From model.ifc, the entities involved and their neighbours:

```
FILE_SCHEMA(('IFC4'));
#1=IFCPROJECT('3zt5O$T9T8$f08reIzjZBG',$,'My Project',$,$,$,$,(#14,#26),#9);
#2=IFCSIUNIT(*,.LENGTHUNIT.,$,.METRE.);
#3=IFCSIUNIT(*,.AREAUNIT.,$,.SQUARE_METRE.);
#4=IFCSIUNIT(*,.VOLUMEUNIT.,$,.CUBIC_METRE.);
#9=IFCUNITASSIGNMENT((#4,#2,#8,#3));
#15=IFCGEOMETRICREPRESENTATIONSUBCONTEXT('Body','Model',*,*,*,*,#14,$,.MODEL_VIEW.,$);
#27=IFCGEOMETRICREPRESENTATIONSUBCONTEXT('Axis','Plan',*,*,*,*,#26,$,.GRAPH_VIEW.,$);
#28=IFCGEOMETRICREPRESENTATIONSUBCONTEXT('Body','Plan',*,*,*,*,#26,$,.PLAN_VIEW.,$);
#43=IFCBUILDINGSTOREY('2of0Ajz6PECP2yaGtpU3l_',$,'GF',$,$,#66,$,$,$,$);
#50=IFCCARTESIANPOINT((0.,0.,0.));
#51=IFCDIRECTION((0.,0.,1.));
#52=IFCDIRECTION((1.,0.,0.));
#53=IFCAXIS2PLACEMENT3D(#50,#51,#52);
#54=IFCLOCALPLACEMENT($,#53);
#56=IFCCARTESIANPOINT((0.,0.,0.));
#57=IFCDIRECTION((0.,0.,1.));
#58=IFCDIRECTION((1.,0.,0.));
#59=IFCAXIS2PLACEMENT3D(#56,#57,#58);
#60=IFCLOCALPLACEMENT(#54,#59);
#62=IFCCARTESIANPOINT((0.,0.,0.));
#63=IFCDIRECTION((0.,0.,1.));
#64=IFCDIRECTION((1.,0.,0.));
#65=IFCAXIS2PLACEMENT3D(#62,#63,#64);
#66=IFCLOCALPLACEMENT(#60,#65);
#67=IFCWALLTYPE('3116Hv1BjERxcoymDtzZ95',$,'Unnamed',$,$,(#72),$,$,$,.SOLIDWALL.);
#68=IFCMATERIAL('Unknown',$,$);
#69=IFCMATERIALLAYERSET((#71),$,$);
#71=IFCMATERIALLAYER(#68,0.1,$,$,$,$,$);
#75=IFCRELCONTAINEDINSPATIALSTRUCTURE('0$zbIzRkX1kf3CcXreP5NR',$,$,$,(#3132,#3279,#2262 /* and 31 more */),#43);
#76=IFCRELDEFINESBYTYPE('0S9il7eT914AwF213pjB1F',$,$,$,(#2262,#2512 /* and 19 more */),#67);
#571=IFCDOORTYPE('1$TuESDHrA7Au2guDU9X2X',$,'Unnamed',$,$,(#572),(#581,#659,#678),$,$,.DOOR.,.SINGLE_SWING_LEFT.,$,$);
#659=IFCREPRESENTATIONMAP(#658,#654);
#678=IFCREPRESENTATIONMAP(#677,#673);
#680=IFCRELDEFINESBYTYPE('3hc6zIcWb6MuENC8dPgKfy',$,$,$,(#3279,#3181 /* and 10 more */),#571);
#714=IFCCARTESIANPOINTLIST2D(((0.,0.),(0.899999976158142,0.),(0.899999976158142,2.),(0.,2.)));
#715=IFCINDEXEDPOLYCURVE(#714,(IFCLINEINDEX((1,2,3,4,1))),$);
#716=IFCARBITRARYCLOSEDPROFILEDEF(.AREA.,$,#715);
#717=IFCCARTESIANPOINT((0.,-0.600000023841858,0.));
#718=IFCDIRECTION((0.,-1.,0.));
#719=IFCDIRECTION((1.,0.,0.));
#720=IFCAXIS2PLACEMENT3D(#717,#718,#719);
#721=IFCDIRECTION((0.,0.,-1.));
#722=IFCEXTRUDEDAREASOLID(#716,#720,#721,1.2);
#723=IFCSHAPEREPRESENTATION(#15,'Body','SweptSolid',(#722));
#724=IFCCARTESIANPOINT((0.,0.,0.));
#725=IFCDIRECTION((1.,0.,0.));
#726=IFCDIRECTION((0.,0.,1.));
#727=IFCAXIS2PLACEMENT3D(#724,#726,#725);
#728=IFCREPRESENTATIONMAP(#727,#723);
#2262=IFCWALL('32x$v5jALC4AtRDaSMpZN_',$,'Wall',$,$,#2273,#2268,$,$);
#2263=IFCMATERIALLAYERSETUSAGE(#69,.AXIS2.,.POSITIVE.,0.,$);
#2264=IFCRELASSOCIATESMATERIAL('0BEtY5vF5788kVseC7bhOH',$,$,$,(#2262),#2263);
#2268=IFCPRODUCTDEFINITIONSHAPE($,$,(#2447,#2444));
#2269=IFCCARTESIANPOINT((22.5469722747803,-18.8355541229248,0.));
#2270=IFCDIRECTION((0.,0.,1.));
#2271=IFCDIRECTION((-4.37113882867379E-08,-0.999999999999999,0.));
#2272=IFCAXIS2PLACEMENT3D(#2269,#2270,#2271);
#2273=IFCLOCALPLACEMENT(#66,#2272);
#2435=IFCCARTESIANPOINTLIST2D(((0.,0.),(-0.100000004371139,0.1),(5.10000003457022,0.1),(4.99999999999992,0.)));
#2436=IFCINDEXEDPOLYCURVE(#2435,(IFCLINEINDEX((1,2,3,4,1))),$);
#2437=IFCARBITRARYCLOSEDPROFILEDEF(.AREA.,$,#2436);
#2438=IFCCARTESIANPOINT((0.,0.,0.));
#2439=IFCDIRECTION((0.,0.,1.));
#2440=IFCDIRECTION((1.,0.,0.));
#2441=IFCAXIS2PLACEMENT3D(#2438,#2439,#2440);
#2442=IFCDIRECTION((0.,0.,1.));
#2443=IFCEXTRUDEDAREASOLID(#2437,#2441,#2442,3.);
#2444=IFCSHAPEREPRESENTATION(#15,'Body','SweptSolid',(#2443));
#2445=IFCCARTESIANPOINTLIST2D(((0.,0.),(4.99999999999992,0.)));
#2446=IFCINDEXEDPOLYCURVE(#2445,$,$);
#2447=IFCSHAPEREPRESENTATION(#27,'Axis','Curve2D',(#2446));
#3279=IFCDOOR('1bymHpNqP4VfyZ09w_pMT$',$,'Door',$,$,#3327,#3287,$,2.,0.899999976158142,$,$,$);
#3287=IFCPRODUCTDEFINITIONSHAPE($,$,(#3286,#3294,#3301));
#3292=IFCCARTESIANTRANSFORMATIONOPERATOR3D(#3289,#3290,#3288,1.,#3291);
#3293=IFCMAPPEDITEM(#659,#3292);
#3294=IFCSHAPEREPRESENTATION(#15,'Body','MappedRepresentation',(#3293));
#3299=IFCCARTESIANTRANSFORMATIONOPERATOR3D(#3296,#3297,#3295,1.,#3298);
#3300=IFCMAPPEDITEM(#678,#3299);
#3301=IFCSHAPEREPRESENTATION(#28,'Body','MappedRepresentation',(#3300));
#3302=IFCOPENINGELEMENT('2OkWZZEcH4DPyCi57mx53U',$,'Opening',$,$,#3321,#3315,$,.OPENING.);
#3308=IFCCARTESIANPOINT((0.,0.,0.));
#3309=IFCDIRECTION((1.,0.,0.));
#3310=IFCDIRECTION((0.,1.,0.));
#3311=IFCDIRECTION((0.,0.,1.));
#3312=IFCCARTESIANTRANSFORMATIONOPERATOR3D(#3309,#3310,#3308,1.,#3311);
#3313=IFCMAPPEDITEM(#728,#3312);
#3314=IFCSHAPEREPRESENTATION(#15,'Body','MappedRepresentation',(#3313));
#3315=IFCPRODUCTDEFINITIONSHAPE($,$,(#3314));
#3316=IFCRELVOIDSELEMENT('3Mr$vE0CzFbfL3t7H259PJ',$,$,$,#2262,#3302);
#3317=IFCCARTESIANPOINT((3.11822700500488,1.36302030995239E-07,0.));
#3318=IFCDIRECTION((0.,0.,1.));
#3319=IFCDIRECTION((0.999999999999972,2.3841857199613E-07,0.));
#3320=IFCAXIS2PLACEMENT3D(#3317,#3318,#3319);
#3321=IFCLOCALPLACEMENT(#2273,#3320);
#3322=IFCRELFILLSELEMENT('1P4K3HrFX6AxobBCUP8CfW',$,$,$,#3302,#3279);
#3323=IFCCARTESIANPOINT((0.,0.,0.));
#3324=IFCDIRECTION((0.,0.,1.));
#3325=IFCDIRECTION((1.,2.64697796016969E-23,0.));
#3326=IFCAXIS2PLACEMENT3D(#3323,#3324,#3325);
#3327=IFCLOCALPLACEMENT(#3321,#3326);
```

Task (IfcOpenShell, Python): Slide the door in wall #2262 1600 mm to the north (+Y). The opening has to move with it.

```python
import ifcopenshell
import ifcopenshell.api.geometry
import ifcopenshell.util.placement
import ifcopenshell.util.unit

model = ifcopenshell.open("model.ifc")
unit_scale = ifcopenshell.util.unit.calculate_unit_scale(model)

door = model.by_id(3279)
opening = door.FillsVoids[0].RelatingOpeningElement
wall = opening.VoidsElements[0].RelatingBuildingElement

wall_matrix = ifcopenshell.util.placement.get_local_placement(wall.ObjectPlacement)
shift = wall_matrix[:3, 0] * -1.6 / unit_scale
before = ifcopenshell.util.placement.get_local_placement(door.ObjectPlacement)[:3, 3].copy()

# The door is placed relative to its opening, so it follows when the opening moves.
matrix = ifcopenshell.util.placement.get_local_placement(opening.ObjectPlacement)
matrix[:3, 3] += shift
ifcopenshell.api.geometry.edit_object_placement(
    model, product=opening, matrix=matrix, is_si=False, should_transform_children=True
)

after = ifcopenshell.util.placement.get_local_placement(door.ObjectPlacement)[:3, 3]
print("door moved by", (after - before).round(3) + 0.0)

model.write("model_updated.ifc")
```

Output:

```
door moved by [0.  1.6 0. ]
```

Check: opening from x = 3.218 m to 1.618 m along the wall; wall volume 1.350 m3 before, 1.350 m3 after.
